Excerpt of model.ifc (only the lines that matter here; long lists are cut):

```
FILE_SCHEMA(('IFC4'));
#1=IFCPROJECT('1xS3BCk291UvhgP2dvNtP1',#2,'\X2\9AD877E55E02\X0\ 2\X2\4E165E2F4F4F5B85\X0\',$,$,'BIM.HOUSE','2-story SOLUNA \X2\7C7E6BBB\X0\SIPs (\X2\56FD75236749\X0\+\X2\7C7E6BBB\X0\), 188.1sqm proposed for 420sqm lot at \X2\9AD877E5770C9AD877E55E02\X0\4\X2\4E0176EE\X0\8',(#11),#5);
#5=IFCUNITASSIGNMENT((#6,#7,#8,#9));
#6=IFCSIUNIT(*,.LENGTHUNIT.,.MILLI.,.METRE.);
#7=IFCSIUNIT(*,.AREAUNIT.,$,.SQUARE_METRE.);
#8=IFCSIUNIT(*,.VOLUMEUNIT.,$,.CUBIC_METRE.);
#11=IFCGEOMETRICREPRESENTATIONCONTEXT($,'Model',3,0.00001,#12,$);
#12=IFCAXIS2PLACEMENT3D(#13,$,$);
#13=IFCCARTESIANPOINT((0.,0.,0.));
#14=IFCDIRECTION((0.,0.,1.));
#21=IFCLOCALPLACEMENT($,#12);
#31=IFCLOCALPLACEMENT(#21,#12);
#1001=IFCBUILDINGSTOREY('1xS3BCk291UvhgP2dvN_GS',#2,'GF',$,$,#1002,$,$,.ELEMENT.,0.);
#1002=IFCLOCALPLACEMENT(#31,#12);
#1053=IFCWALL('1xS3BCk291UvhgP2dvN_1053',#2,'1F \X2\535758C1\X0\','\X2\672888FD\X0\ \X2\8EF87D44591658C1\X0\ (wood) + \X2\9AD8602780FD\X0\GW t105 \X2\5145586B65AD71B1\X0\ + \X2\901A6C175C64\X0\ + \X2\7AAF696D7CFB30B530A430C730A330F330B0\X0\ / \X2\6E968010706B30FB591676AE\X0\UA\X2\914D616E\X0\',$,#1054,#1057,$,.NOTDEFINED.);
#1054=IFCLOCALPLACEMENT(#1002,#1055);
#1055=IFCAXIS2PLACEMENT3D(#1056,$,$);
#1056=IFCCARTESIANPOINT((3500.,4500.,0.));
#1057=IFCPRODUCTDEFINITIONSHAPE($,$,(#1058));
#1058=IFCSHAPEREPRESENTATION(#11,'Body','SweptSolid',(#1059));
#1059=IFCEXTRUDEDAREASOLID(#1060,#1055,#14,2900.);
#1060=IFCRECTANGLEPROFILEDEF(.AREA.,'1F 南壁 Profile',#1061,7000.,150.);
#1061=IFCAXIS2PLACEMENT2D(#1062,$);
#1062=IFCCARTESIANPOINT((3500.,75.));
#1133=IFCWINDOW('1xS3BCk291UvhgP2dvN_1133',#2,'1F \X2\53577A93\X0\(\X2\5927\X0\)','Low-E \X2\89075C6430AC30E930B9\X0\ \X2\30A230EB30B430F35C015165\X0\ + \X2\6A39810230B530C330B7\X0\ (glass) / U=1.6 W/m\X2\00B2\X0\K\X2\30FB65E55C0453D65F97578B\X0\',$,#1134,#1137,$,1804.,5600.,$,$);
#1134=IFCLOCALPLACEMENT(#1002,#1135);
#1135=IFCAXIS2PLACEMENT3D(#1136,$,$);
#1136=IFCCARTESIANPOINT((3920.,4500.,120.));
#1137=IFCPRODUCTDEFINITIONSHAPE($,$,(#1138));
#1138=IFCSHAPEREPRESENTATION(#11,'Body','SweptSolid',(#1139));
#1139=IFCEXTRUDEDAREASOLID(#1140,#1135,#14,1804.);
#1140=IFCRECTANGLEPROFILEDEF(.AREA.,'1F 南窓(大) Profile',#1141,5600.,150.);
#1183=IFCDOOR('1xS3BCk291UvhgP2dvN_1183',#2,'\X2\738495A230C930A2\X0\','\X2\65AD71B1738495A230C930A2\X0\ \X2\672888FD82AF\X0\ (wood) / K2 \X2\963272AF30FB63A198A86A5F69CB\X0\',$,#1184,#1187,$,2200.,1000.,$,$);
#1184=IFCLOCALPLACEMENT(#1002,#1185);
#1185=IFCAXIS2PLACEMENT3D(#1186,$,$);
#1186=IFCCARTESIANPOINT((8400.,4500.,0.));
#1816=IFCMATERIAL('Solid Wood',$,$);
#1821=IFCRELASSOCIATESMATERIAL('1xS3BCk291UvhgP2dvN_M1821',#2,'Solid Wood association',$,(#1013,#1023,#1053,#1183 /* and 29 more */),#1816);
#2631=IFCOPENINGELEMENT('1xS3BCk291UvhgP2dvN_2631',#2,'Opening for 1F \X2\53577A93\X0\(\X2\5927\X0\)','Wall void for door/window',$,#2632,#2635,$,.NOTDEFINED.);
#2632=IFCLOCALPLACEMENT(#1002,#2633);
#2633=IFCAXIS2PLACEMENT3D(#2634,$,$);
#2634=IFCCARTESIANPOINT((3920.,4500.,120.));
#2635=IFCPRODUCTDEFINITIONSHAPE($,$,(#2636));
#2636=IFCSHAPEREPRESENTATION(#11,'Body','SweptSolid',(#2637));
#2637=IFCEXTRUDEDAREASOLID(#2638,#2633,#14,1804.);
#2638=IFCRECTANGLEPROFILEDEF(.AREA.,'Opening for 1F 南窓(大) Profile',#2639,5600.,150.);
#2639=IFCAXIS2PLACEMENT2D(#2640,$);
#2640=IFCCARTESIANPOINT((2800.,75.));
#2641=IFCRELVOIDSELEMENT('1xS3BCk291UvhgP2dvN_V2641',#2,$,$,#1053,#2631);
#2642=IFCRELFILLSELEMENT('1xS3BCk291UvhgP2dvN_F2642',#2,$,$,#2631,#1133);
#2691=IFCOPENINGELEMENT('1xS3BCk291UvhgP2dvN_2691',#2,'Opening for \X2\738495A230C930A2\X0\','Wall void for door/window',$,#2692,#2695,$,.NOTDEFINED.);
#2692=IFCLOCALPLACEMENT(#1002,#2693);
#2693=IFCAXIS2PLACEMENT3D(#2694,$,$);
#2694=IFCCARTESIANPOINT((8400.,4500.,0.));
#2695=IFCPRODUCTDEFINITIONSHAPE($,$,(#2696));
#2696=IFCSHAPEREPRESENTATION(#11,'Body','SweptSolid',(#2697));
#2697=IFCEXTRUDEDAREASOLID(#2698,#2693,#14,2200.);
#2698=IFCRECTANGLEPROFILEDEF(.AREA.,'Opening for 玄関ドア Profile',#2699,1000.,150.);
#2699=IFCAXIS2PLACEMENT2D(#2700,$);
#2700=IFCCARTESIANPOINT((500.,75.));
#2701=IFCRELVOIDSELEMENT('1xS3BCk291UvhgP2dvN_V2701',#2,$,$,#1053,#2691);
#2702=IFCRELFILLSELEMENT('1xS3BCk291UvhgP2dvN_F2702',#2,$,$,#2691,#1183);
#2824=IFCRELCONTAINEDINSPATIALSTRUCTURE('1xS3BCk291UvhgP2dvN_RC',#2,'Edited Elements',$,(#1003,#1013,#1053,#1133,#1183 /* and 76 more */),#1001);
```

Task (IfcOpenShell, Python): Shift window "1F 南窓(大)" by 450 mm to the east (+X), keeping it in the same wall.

```python
import ifcopenshell
import ifcopenshell.api.geometry
import ifcopenshell.util.placement
import ifcopenshell.util.unit

model = ifcopenshell.open("model.ifc")
unit_scale = ifcopenshell.util.unit.calculate_unit_scale(model)

window = model.by_guid("1xS3BCk291UvhgP2dvN_1133")
opening = window.FillsVoids[0].RelatingOpeningElement
wall = opening.VoidsElements[0].RelatingBuildingElement

wall_matrix = ifcopenshell.util.placement.get_local_placement(wall.ObjectPlacement)
shift = wall_matrix[:3, 0] * 0.45 / unit_scale
before = ifcopenshell.util.placement.get_local_placement(window.ObjectPlacement)[:3, 3].copy()

# The window is not placed relative to its opening, so move both.
for product in (opening, window):
    matrix = ifcopenshell.util.placement.get_local_placement(product.ObjectPlacement)
    matrix[:3, 3] += shift
    ifcopenshell.api.geometry.edit_object_placement(model, product=product, matrix=matrix, is_si=False)

after = ifcopenshell.util.placement.get_local_placement(window.ObjectPlacement)[:3, 3]
print("window moved by", (after - before).round(3) + 0.0)

model.write("model_v2.ifc")
```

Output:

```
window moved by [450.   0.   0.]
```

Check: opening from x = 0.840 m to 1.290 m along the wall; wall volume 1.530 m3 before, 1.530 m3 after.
